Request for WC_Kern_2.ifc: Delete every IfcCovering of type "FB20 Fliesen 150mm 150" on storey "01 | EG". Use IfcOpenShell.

First a look at what the model holds.

```python
import ifcopenshell
import ifcopenshell.util.element

model = ifcopenshell.open("WC_Kern_2.ifc")
print(model.schema)
storey = next(s for s in model.by_type("IfcBuildingStorey") if s.Name == "01 | EG")
coverings = [e for e in ifcopenshell.util.element.get_decomposition(storey) if e.is_a("IfcCovering")]
seen = {}
for e in coverings:
    element_type = ifcopenshell.util.element.get_type(e)
    name = element_type.Name if element_type not in (None, e) else None
    seen[name] = seen.get(name, 0) + 1
for name, count in sorted(seen.items(), key=str):
    print(count, "x", name)
```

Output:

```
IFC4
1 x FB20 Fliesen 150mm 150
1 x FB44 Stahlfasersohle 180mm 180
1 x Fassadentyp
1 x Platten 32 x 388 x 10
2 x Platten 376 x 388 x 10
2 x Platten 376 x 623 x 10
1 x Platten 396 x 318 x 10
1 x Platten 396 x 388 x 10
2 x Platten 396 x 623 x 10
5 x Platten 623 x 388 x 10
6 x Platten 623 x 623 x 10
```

```python
import ifcopenshell
import ifcopenshell.api.root
import ifcopenshell.util.element

model = ifcopenshell.open("WC_Kern_2.ifc")

storey = next(s for s in model.by_type("IfcBuildingStorey") if s.Name == "01 | EG")
coverings = [e for e in ifcopenshell.util.element.get_decomposition(storey) if e.is_a("IfcCovering")]
targets = [e for e in coverings if (t := ifcopenshell.util.element.get_type(e)) not in (None, e) and t.Name == "FB20 Fliesen 150mm 150"]

for e in targets:
    ifcopenshell.api.root.remove_product(model, product=e)
print(len(targets), "removed")

model.write("WC_Kern_2_updated.ifc")
```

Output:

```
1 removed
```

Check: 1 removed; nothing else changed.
